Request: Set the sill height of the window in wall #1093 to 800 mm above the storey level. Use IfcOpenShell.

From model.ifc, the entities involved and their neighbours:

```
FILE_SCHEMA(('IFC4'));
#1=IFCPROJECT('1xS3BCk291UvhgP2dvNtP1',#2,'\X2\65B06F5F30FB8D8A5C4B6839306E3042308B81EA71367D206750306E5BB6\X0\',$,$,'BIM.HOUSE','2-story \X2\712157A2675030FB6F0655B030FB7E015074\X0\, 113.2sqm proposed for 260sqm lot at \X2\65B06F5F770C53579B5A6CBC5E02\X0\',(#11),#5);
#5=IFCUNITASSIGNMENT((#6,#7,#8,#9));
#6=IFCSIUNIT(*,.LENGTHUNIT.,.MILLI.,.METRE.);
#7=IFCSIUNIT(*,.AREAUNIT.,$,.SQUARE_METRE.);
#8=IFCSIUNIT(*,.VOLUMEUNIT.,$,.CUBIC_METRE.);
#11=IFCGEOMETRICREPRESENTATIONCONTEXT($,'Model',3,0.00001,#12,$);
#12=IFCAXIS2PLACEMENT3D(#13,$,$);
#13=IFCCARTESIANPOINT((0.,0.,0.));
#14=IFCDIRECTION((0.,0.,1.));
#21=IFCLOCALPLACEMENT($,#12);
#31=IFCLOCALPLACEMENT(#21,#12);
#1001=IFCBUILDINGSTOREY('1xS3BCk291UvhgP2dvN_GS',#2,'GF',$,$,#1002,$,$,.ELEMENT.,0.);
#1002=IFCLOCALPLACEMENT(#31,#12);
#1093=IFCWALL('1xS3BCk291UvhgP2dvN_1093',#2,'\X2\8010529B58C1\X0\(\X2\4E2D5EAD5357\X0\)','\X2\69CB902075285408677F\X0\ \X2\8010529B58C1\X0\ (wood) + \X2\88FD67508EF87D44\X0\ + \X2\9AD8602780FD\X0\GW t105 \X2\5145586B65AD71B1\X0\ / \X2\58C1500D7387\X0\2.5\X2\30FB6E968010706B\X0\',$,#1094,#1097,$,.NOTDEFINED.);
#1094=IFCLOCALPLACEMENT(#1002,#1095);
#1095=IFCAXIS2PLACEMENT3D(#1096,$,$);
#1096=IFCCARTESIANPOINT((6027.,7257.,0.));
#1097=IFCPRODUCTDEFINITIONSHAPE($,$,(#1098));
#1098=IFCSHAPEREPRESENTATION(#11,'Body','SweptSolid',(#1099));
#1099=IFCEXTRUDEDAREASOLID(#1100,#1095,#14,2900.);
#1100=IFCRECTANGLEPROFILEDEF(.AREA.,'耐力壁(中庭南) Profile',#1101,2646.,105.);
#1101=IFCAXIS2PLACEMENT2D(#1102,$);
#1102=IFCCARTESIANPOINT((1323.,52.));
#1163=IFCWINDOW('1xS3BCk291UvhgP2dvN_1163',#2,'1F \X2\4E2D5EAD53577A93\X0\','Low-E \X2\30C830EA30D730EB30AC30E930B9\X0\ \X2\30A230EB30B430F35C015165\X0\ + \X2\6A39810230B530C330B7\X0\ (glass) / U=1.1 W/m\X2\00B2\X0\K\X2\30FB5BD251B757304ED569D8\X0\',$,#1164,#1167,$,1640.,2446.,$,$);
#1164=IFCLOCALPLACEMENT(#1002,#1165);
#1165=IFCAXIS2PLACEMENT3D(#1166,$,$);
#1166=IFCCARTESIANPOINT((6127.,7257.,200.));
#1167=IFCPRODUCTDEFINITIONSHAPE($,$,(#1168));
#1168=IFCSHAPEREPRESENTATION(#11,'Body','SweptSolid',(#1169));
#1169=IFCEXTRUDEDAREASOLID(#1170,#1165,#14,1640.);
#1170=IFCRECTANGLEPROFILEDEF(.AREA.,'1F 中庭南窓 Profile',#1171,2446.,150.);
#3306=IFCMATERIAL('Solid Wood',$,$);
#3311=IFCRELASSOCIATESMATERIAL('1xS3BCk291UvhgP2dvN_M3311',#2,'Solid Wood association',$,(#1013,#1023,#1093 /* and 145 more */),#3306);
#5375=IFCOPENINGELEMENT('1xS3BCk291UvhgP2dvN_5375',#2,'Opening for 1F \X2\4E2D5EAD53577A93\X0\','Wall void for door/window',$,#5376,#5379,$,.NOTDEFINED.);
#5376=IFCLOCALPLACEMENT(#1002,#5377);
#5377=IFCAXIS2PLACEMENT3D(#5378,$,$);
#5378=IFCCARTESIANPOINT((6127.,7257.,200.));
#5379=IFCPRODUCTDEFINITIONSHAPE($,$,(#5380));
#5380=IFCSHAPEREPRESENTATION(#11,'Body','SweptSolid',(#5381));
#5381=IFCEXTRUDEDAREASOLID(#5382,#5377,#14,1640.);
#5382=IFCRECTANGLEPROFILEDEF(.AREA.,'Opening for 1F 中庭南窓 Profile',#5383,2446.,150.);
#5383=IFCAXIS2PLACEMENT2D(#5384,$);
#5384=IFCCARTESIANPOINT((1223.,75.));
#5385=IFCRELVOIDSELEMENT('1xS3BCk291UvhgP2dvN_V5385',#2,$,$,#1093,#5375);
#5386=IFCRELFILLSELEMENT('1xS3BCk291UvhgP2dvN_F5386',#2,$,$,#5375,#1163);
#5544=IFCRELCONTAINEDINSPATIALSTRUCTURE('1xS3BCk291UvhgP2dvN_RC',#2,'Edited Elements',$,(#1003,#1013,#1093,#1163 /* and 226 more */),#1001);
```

```python
import numpy as np
import ifcopenshell
import ifcopenshell.api.geometry
import ifcopenshell.geom
import ifcopenshell.util.element
import ifcopenshell.util.placement
import ifcopenshell.util.shape
import ifcopenshell.util.unit

model = ifcopenshell.open("model.ifc")
unit_scale = ifcopenshell.util.unit.calculate_unit_scale(model)

window = model.by_guid("1xS3BCk291UvhgP2dvN_1163")
opening = window.FillsVoids[0].RelatingOpeningElement
storey = ifcopenshell.util.element.get_container(window, ifc_class="IfcBuildingStorey")
level = ifcopenshell.util.placement.get_local_placement(storey.ObjectPlacement)[2, 3]

# The opening's origin need not be at the sill, so measure its lowest point.
shape = ifcopenshell.geom.create_shape(ifcopenshell.geom.settings(), opening)
bottom = ifcopenshell.util.shape.get_shape_bottom_elevation(shape, shape.geometry) / unit_scale
dz = level + 0.8 / unit_scale - bottom

shift = np.array([0.0, 0.0, dz])
# The window is not placed relative to its opening, so move both.
for product in (opening, window):
    matrix = ifcopenshell.util.placement.get_local_placement(product.ObjectPlacement)
    matrix[:3, 3] += shift
    ifcopenshell.api.geometry.edit_object_placement(model, product=product, matrix=matrix, is_si=False)

print(f"moved by {dz * unit_scale:+.3f} m")

model.write("model_v2.ifc")
```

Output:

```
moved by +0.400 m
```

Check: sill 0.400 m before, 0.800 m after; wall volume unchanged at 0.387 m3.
